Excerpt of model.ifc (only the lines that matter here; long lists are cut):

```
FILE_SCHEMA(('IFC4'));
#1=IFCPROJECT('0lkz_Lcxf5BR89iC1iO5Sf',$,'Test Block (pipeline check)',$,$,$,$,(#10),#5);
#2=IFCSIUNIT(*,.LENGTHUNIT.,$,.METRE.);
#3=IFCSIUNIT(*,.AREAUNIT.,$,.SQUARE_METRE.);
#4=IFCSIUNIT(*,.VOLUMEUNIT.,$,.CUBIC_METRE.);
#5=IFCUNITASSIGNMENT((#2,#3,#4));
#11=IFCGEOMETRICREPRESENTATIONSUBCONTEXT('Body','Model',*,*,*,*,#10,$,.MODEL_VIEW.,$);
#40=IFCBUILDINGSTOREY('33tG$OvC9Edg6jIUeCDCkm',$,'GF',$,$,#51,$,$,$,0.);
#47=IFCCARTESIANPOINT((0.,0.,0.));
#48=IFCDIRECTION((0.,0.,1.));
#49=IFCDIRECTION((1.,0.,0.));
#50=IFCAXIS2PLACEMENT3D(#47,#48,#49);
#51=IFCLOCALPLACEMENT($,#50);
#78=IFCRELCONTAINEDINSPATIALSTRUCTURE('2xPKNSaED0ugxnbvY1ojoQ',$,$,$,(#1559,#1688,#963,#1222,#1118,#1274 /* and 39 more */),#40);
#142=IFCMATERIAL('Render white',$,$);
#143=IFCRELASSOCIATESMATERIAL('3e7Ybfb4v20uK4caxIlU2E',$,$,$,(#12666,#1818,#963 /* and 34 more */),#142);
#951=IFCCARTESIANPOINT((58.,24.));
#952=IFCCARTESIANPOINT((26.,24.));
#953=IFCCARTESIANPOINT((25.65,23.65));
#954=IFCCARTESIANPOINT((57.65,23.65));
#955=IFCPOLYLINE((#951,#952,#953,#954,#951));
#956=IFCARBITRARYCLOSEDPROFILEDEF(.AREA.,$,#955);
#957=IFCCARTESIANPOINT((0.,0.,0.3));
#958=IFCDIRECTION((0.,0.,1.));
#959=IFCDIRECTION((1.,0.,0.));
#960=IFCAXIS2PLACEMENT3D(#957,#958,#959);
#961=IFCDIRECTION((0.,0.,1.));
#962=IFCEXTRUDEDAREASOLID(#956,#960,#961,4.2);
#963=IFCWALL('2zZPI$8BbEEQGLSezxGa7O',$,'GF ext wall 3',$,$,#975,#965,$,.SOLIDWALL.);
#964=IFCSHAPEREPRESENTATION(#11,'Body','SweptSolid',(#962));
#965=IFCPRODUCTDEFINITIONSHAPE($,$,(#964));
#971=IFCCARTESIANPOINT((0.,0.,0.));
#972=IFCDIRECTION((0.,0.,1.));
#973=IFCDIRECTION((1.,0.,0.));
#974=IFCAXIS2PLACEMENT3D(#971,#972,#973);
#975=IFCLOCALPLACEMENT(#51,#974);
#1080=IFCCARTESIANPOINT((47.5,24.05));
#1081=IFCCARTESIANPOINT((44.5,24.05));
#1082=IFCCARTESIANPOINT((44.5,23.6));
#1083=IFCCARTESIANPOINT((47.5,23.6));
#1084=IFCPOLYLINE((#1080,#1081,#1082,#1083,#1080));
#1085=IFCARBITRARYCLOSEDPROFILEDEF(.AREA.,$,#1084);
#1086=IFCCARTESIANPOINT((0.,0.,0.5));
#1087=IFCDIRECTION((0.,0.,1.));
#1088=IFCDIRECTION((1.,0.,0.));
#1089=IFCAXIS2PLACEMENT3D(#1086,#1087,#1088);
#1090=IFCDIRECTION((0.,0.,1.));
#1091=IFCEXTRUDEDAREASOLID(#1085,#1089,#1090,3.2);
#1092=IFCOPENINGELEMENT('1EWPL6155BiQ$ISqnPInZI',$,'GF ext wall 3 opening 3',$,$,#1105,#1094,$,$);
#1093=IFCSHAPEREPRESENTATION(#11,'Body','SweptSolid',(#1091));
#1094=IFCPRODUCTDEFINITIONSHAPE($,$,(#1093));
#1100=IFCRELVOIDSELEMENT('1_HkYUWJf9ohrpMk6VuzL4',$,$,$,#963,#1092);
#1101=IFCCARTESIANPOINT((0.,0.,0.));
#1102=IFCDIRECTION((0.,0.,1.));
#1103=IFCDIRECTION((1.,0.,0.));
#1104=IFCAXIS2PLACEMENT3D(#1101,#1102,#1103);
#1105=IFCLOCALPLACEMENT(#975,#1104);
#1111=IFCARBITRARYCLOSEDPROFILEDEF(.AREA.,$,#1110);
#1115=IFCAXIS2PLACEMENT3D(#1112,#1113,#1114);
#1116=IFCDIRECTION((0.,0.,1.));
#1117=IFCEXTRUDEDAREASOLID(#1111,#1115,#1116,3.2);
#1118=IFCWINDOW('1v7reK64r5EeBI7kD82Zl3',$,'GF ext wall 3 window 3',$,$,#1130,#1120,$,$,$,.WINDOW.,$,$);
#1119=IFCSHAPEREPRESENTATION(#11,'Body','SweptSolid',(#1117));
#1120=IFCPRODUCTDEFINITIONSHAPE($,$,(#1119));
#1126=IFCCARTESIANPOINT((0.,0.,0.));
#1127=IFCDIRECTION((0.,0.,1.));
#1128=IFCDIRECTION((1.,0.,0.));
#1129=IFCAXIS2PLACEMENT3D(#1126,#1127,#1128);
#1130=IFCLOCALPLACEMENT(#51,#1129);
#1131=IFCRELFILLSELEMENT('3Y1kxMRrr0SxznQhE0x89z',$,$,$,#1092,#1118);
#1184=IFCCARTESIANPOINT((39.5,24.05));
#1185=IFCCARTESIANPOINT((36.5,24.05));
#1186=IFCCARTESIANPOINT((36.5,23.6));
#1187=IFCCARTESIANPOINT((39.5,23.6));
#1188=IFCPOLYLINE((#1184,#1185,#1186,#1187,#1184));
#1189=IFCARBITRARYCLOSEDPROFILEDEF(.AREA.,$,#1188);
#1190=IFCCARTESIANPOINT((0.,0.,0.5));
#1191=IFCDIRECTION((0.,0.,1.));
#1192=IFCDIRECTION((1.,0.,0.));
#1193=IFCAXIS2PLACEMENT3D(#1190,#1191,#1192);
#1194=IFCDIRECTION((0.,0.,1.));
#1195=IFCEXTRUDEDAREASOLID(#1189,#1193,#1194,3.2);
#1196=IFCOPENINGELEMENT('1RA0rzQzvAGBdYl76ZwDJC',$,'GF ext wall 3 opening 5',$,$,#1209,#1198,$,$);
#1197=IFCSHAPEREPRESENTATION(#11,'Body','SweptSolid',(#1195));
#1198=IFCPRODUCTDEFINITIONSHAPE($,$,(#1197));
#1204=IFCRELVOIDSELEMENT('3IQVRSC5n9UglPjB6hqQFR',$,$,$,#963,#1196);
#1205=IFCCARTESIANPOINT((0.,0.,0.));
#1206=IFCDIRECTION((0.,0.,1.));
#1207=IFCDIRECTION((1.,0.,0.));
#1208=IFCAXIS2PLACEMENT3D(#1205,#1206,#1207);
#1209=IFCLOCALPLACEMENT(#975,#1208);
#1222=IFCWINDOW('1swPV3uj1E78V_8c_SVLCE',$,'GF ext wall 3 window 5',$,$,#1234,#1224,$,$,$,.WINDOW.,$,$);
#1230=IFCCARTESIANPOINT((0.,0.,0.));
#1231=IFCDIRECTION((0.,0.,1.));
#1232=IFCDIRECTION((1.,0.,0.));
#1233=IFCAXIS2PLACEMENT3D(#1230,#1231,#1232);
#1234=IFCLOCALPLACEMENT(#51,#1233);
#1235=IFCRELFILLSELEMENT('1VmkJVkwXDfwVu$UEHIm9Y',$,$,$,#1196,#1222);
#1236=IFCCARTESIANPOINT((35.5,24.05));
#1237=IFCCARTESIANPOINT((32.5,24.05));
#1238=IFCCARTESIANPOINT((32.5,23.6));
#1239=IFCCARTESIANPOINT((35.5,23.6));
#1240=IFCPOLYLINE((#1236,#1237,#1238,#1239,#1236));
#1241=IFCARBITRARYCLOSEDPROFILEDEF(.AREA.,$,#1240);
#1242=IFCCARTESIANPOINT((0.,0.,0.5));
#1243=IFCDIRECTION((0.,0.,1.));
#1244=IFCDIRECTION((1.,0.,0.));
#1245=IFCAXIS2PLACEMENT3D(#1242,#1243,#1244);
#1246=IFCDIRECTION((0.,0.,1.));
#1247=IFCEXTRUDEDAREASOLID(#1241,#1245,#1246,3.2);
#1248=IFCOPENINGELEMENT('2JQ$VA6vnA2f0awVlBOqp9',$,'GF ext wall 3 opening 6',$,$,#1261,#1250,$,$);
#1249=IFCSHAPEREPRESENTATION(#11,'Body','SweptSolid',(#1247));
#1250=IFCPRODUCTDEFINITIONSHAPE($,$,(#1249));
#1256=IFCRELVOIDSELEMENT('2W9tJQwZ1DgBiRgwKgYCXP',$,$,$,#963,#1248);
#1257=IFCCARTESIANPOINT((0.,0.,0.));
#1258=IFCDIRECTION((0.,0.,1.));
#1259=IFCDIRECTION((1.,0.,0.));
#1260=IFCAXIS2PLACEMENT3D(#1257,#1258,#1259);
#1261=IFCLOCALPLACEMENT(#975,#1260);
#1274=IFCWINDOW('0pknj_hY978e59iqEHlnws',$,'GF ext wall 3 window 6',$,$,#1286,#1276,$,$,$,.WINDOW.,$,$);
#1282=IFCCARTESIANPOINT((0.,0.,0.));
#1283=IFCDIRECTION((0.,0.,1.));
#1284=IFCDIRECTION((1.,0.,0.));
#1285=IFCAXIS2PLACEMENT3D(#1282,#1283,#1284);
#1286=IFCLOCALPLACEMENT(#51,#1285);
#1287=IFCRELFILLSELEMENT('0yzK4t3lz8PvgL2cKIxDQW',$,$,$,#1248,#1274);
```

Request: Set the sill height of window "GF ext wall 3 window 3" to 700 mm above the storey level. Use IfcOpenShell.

```python
import numpy as np
import ifcopenshell
import ifcopenshell.api.geometry
import ifcopenshell.geom
import ifcopenshell.util.element
import ifcopenshell.util.placement
import ifcopenshell.util.shape
import ifcopenshell.util.unit

model = ifcopenshell.open("model.ifc")
unit_scale = ifcopenshell.util.unit.calculate_unit_scale(model)

window = model.by_id(1118)
opening = window.FillsVoids[0].RelatingOpeningElement
storey = ifcopenshell.util.element.get_container(window, ifc_class="IfcBuildingStorey")
level = ifcopenshell.util.placement.get_local_placement(storey.ObjectPlacement)[2, 3]

# The opening's origin need not be at the sill, so measure its lowest point.
shape = ifcopenshell.geom.create_shape(ifcopenshell.geom.settings(), opening)
bottom = ifcopenshell.util.shape.get_shape_bottom_elevation(shape, shape.geometry) / unit_scale
dz = level + 0.7 / unit_scale - bottom

shift = np.array([0.0, 0.0, dz])
# The window is not placed relative to its opening, so move both.
for product in (opening, window):
    matrix = ifcopenshell.util.placement.get_local_placement(product.ObjectPlacement)
    matrix[:3, 3] += shift
    ifcopenshell.api.geometry.edit_object_placement(model, product=product, matrix=matrix, is_si=False)

print(f"moved by {dz * unit_scale:+.3f} m")

model.write("model-out.ifc")
```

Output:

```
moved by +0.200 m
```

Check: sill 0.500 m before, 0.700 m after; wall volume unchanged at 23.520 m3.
